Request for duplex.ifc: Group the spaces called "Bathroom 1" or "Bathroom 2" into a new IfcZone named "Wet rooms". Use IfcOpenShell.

First a look at what the model holds.

```python
import ifcopenshell

model = ifcopenshell.open("duplex.ifc")
print(model.schema)
seen = {}
for space in model.by_type("IfcSpace"):
    seen[space.LongName] = seen.get(space.LongName, 0) + 1
for name, count in sorted(seen.items(), key=str):
    print(count, "x", name)
print("zones:", [z.Name for z in model.by_type("IfcZone")][:20])
```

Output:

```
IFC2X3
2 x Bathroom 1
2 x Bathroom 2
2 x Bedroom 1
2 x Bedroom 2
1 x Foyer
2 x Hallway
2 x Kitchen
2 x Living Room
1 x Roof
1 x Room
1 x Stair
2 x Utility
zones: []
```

```python
import ifcopenshell
import ifcopenshell.api.group
import ifcopenshell.api.root

model = ifcopenshell.open("duplex.ifc")

names = {"Bathroom 1", "Bathroom 2"}
spaces = [s for s in model.by_type("IfcSpace") if s.LongName in names]

zone = ifcopenshell.api.root.create_entity(model, ifc_class="IfcZone", name="Wet rooms")
ifcopenshell.api.group.assign_group(model, products=spaces, group=zone)
print(len(spaces), "spaces in", zone.Name)

model.write("duplex-out.ifc")
```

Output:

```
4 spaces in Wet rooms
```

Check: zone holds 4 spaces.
